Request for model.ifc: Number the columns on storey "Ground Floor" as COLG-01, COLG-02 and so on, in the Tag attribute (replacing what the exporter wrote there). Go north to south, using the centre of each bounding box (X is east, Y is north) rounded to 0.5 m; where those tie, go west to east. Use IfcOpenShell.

First a look at what the model holds.

```python
import ifcopenshell
import ifcopenshell.util.element
import ifcopenshell.util.placement

model = ifcopenshell.open("model.ifc")
print(model.schema)
storey = next(s for s in model.by_type("IfcBuildingStorey") if s.Name == "Ground Floor")
columns = [e for e in ifcopenshell.util.element.get_decomposition(storey) if e.is_a("IfcColumn")]
for e in sorted(columns, key=lambda e: e.id()):
    origin = ifcopenshell.util.placement.get_local_placement(e.ObjectPlacement)[:3, 3]
    print(e.id(), e.Tag, e.Name, origin.round(2) + 0.0, sep=" | ")
```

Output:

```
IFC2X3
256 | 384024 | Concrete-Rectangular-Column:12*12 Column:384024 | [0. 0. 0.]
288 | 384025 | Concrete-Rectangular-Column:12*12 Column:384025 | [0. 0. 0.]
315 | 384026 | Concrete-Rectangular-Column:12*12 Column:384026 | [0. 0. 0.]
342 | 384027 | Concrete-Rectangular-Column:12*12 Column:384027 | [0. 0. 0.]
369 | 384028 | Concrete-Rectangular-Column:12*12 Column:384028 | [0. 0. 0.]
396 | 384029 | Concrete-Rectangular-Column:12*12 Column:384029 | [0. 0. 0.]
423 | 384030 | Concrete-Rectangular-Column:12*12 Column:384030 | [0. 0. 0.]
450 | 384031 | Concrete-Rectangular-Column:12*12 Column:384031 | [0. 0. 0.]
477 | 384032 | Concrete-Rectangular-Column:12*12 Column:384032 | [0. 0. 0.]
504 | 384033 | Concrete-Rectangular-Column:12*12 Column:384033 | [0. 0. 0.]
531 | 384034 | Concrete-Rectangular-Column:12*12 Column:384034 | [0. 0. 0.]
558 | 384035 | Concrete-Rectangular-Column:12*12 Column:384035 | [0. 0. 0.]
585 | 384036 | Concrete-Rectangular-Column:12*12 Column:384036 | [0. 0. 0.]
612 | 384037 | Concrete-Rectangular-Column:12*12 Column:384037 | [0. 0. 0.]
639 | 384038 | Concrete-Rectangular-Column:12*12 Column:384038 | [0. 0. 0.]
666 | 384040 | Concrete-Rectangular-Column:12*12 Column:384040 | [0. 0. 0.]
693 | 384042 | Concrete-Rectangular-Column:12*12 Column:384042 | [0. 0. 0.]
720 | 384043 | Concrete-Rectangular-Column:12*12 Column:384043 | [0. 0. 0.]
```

```python
import ifcopenshell
import ifcopenshell.geom
import ifcopenshell.util.element
import ifcopenshell.util.shape

model = ifcopenshell.open("model.ifc")
settings = ifcopenshell.geom.settings()
settings.set("use-world-coords", True)


def centre(element):
    shape = ifcopenshell.geom.create_shape(settings, element)
    return ifcopenshell.util.shape.get_bbox_centroid(shape.geometry)


storey = next(s for s in model.by_type("IfcBuildingStorey") if s.Name == "Ground Floor")
columns = [e for e in ifcopenshell.util.element.get_decomposition(storey) if e.is_a("IfcColumn")]

# Insertion points can sit at a corner or the storey origin, so sort by the geometry (in metres).
centres = {e: centre(e) for e in columns}
columns.sort(key=lambda e: (-round(centres[e][1] / 0.5), centres[e][0]))

for i, e in enumerate(columns, start=1):
    number = f"COLG-{i:02d}"
    e.Tag = number
    print(e.id(), number)

model.write("model_edited.ifc")
```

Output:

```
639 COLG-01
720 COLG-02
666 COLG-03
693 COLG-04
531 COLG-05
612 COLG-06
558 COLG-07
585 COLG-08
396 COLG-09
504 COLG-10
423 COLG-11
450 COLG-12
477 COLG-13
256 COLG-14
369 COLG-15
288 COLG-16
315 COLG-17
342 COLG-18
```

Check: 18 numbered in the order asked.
